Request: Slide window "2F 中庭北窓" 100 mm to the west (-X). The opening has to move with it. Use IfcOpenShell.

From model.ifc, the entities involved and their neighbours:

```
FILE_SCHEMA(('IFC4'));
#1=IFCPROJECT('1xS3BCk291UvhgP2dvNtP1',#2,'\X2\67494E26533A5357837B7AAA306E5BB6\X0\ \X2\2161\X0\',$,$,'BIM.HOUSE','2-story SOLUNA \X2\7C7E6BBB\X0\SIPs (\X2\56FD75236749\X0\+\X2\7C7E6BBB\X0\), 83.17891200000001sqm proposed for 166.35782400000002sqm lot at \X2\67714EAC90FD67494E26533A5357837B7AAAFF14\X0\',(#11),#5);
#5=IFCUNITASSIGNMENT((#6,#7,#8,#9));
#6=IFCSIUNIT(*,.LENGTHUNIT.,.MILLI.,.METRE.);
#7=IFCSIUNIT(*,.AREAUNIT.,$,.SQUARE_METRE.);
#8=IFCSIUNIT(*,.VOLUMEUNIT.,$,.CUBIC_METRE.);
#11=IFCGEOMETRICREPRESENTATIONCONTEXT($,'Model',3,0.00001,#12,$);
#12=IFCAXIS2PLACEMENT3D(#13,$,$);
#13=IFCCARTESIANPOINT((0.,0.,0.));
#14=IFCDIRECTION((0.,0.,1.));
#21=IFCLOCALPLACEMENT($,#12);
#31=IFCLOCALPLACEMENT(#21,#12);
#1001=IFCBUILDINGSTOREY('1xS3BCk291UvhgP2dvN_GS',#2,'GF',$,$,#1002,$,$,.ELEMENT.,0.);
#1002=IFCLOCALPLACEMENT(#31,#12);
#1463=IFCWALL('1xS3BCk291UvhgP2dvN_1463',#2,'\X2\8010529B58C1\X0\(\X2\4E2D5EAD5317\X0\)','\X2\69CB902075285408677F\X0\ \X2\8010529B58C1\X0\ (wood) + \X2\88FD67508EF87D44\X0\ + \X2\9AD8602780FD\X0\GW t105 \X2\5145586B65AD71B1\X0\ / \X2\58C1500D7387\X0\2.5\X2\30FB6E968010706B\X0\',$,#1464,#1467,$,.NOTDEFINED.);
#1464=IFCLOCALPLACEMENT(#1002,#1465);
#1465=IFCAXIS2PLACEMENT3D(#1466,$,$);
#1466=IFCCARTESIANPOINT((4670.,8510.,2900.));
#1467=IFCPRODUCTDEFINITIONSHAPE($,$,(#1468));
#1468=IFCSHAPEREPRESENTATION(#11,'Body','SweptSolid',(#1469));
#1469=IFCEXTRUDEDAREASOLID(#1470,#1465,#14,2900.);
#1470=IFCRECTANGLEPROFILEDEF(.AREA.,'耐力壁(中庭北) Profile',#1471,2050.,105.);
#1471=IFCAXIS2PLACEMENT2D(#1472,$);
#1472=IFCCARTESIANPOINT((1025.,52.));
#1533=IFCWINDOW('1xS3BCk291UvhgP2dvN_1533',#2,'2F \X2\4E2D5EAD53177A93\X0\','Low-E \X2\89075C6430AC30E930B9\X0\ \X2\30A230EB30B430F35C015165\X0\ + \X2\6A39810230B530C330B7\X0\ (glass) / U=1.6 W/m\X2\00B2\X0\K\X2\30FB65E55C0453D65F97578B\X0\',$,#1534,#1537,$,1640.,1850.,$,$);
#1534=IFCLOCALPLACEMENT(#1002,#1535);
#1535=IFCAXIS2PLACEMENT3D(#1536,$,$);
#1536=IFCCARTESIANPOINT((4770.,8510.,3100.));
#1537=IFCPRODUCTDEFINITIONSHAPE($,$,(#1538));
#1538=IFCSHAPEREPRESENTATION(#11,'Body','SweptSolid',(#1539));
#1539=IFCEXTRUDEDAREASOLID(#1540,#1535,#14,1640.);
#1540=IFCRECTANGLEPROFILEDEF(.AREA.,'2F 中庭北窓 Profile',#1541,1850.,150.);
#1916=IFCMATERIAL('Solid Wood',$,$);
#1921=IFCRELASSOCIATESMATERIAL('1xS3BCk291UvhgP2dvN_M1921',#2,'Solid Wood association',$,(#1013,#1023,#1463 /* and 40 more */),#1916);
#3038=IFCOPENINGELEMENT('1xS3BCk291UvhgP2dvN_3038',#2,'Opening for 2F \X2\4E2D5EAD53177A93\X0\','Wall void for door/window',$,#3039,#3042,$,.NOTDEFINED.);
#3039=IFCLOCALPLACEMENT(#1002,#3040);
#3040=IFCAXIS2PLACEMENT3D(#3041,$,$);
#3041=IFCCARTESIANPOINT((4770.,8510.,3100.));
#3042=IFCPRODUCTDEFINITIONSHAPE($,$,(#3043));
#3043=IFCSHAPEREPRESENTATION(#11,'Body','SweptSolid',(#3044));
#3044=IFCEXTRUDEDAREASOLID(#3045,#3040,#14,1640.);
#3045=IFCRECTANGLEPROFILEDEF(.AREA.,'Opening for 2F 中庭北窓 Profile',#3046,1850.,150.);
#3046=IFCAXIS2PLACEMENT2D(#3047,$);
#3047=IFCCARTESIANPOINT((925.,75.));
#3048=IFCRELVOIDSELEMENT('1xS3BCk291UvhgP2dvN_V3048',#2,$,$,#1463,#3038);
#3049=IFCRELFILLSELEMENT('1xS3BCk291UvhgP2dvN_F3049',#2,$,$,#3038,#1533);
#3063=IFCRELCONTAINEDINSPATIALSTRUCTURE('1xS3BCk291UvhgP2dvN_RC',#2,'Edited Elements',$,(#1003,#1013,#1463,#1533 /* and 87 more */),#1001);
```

```python
import ifcopenshell
import ifcopenshell.api.geometry
import ifcopenshell.util.placement
import ifcopenshell.util.unit

model = ifcopenshell.open("model.ifc")
unit_scale = ifcopenshell.util.unit.calculate_unit_scale(model)

window = model.by_guid("1xS3BCk291UvhgP2dvN_1533")
opening = window.FillsVoids[0].RelatingOpeningElement
wall = opening.VoidsElements[0].RelatingBuildingElement

wall_matrix = ifcopenshell.util.placement.get_local_placement(wall.ObjectPlacement)
shift = wall_matrix[:3, 0] * -0.1 / unit_scale
before = ifcopenshell.util.placement.get_local_placement(window.ObjectPlacement)[:3, 3].copy()

# The window is not placed relative to its opening, so move both.
for product in (opening, window):
    matrix = ifcopenshell.util.placement.get_local_placement(product.ObjectPlacement)
    matrix[:3, 3] += shift
    ifcopenshell.api.geometry.edit_object_placement(model, product=product, matrix=matrix, is_si=False)

after = ifcopenshell.util.placement.get_local_placement(window.ObjectPlacement)[:3, 3]
print("window moved by", (after - before).round(3) + 0.0)

model.write("model_rev.ifc")
```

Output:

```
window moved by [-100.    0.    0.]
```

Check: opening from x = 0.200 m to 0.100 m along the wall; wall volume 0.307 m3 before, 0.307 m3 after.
